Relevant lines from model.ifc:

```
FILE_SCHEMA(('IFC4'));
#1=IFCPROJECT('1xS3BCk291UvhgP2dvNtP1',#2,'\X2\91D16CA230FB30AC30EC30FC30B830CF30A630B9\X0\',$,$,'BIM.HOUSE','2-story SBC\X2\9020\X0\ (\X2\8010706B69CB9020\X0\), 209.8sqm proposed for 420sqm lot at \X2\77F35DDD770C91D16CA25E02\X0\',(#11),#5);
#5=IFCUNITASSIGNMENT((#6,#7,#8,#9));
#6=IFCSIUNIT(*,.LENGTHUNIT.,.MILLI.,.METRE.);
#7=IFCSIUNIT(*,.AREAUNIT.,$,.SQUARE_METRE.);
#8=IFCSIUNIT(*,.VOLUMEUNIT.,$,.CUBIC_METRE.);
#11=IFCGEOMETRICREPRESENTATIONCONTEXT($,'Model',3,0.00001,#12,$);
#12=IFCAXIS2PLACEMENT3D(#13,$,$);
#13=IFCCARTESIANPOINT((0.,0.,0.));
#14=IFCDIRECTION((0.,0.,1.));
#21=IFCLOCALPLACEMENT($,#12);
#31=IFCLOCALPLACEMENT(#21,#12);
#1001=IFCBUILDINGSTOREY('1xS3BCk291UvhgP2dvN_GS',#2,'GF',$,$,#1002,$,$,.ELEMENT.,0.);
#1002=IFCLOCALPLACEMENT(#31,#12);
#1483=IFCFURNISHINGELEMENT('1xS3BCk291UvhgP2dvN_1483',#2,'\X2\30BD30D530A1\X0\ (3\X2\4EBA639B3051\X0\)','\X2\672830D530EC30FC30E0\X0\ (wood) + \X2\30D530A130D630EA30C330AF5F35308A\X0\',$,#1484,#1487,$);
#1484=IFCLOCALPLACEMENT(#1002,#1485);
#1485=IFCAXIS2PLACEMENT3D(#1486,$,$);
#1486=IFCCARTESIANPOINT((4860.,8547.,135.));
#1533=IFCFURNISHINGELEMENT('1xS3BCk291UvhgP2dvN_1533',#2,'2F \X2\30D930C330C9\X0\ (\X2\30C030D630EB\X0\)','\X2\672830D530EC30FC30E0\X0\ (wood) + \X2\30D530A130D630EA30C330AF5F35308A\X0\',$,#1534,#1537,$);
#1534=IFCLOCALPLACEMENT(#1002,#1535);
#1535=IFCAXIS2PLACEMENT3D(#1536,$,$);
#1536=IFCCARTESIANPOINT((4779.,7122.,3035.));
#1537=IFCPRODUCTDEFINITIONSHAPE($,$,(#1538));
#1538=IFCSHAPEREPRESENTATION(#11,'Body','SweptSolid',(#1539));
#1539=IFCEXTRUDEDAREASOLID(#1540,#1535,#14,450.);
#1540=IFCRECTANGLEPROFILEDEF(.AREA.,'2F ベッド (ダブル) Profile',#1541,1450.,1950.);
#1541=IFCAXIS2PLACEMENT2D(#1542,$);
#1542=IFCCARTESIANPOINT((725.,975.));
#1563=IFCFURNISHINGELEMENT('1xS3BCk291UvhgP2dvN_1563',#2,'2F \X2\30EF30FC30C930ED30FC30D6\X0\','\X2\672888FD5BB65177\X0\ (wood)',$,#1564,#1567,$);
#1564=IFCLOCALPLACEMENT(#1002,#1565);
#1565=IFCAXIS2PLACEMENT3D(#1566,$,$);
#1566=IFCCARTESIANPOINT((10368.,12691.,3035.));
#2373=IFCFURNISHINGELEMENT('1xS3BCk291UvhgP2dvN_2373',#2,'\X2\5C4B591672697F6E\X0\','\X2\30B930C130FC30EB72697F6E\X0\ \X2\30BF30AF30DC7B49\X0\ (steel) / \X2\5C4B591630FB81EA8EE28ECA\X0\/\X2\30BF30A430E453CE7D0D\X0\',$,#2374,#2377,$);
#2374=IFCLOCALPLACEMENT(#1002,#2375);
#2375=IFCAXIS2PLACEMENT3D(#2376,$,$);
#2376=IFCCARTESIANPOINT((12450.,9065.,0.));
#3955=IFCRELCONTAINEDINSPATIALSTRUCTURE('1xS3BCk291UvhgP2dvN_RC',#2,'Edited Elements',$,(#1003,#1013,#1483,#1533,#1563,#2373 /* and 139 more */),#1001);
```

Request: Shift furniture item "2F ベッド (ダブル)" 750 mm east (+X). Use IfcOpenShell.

```python
import ifcopenshell
import ifcopenshell.api.geometry
import ifcopenshell.util.placement
import ifcopenshell.util.unit

model = ifcopenshell.open("model.ifc")
unit_scale = ifcopenshell.util.unit.calculate_unit_scale(model)

item = model.by_id(1533)
matrix = ifcopenshell.util.placement.get_local_placement(item.ObjectPlacement)
matrix[0, 3] += 0.75 / unit_scale
ifcopenshell.api.geometry.edit_object_placement(model, product=item, matrix=matrix, is_si=False)

print(ifcopenshell.util.placement.get_local_placement(item.ObjectPlacement).round(3) + 0.0)

model.write("model_updated.ifc")
```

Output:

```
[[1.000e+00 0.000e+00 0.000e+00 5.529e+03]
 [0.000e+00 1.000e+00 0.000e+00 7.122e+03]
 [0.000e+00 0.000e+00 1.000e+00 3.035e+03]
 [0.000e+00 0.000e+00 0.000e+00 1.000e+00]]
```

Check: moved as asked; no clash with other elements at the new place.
